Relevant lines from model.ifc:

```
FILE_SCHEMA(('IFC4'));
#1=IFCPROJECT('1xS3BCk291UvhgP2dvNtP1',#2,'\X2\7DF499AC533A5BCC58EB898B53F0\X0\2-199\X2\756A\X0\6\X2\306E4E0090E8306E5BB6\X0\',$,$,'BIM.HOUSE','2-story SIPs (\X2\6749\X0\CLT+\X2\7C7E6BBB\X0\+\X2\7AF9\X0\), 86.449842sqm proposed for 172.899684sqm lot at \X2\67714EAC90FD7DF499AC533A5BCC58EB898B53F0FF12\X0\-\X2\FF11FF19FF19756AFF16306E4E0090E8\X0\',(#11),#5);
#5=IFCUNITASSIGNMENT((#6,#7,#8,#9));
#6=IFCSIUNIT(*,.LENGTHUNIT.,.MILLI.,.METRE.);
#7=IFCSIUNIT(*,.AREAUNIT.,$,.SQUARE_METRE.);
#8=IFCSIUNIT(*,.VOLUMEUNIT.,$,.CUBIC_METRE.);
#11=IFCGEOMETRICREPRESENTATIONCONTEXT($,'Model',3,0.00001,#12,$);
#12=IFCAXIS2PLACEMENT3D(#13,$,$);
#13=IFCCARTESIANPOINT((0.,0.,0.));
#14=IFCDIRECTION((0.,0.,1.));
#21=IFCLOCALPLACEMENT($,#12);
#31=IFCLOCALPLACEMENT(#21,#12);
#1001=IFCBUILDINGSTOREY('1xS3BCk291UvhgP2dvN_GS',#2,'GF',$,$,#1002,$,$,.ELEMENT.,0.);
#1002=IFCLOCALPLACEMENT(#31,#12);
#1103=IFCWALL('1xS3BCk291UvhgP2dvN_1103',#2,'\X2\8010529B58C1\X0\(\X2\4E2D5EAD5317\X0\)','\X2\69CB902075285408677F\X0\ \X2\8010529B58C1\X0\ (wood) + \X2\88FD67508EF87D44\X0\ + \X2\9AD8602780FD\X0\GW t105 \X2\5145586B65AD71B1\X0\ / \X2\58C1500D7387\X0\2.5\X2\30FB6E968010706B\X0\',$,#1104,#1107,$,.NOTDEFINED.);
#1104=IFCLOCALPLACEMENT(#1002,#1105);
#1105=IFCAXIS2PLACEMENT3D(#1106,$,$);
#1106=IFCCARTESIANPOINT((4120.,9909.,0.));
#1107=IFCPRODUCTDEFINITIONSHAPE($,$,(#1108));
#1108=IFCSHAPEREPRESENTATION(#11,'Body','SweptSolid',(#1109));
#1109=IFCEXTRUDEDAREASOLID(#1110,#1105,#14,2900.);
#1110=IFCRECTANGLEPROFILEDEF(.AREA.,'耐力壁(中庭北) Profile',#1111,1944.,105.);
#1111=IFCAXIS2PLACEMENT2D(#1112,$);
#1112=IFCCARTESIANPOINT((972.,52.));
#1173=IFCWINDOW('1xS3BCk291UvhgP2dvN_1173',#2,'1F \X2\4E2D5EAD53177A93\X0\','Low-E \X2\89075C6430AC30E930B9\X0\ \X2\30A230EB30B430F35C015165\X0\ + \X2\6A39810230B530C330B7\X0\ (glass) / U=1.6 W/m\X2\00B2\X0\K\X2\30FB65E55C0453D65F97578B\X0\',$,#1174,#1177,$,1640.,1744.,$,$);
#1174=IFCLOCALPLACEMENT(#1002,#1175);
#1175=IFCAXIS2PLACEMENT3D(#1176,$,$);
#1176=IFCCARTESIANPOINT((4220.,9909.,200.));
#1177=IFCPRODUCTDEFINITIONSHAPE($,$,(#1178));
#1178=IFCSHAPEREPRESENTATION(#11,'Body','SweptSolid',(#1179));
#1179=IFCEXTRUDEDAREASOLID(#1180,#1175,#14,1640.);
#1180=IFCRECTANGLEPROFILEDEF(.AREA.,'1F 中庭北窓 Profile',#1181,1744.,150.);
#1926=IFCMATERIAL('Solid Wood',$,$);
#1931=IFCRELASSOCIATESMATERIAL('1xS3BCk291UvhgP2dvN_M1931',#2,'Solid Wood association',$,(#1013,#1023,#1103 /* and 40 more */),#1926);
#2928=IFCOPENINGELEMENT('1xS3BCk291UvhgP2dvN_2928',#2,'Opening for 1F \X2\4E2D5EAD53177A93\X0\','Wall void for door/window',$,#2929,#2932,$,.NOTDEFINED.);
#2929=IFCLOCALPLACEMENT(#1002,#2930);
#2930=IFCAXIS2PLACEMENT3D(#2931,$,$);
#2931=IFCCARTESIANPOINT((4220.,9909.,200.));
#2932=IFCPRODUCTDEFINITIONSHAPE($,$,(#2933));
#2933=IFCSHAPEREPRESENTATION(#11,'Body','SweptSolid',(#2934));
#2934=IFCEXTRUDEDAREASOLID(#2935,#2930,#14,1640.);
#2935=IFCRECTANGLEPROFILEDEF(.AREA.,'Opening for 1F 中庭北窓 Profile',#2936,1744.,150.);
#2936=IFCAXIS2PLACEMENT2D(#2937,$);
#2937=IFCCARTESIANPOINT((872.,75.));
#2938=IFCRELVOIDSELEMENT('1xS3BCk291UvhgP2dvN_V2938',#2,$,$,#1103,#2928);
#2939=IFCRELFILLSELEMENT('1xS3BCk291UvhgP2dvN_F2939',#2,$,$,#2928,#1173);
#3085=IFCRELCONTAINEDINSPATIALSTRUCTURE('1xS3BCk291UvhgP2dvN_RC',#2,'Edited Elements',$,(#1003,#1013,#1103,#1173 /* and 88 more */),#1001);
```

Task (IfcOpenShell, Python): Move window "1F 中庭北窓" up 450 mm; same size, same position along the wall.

```python
import numpy as np
import ifcopenshell
import ifcopenshell.api.geometry
import ifcopenshell.util.placement
import ifcopenshell.util.unit

model = ifcopenshell.open("model.ifc")
unit_scale = ifcopenshell.util.unit.calculate_unit_scale(model)

window = model.by_id(1173)
opening = window.FillsVoids[0].RelatingOpeningElement
dz = 0.45 / unit_scale

shift = np.array([0.0, 0.0, dz])
# The window is not placed relative to its opening, so move both.
for product in (opening, window):
    matrix = ifcopenshell.util.placement.get_local_placement(product.ObjectPlacement)
    matrix[:3, 3] += shift
    ifcopenshell.api.geometry.edit_object_placement(model, product=product, matrix=matrix, is_si=False)

print(f"moved by {dz * unit_scale:+.3f} m")

model.write("model_edited.ifc")
```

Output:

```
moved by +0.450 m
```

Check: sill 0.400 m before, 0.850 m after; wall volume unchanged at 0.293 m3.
